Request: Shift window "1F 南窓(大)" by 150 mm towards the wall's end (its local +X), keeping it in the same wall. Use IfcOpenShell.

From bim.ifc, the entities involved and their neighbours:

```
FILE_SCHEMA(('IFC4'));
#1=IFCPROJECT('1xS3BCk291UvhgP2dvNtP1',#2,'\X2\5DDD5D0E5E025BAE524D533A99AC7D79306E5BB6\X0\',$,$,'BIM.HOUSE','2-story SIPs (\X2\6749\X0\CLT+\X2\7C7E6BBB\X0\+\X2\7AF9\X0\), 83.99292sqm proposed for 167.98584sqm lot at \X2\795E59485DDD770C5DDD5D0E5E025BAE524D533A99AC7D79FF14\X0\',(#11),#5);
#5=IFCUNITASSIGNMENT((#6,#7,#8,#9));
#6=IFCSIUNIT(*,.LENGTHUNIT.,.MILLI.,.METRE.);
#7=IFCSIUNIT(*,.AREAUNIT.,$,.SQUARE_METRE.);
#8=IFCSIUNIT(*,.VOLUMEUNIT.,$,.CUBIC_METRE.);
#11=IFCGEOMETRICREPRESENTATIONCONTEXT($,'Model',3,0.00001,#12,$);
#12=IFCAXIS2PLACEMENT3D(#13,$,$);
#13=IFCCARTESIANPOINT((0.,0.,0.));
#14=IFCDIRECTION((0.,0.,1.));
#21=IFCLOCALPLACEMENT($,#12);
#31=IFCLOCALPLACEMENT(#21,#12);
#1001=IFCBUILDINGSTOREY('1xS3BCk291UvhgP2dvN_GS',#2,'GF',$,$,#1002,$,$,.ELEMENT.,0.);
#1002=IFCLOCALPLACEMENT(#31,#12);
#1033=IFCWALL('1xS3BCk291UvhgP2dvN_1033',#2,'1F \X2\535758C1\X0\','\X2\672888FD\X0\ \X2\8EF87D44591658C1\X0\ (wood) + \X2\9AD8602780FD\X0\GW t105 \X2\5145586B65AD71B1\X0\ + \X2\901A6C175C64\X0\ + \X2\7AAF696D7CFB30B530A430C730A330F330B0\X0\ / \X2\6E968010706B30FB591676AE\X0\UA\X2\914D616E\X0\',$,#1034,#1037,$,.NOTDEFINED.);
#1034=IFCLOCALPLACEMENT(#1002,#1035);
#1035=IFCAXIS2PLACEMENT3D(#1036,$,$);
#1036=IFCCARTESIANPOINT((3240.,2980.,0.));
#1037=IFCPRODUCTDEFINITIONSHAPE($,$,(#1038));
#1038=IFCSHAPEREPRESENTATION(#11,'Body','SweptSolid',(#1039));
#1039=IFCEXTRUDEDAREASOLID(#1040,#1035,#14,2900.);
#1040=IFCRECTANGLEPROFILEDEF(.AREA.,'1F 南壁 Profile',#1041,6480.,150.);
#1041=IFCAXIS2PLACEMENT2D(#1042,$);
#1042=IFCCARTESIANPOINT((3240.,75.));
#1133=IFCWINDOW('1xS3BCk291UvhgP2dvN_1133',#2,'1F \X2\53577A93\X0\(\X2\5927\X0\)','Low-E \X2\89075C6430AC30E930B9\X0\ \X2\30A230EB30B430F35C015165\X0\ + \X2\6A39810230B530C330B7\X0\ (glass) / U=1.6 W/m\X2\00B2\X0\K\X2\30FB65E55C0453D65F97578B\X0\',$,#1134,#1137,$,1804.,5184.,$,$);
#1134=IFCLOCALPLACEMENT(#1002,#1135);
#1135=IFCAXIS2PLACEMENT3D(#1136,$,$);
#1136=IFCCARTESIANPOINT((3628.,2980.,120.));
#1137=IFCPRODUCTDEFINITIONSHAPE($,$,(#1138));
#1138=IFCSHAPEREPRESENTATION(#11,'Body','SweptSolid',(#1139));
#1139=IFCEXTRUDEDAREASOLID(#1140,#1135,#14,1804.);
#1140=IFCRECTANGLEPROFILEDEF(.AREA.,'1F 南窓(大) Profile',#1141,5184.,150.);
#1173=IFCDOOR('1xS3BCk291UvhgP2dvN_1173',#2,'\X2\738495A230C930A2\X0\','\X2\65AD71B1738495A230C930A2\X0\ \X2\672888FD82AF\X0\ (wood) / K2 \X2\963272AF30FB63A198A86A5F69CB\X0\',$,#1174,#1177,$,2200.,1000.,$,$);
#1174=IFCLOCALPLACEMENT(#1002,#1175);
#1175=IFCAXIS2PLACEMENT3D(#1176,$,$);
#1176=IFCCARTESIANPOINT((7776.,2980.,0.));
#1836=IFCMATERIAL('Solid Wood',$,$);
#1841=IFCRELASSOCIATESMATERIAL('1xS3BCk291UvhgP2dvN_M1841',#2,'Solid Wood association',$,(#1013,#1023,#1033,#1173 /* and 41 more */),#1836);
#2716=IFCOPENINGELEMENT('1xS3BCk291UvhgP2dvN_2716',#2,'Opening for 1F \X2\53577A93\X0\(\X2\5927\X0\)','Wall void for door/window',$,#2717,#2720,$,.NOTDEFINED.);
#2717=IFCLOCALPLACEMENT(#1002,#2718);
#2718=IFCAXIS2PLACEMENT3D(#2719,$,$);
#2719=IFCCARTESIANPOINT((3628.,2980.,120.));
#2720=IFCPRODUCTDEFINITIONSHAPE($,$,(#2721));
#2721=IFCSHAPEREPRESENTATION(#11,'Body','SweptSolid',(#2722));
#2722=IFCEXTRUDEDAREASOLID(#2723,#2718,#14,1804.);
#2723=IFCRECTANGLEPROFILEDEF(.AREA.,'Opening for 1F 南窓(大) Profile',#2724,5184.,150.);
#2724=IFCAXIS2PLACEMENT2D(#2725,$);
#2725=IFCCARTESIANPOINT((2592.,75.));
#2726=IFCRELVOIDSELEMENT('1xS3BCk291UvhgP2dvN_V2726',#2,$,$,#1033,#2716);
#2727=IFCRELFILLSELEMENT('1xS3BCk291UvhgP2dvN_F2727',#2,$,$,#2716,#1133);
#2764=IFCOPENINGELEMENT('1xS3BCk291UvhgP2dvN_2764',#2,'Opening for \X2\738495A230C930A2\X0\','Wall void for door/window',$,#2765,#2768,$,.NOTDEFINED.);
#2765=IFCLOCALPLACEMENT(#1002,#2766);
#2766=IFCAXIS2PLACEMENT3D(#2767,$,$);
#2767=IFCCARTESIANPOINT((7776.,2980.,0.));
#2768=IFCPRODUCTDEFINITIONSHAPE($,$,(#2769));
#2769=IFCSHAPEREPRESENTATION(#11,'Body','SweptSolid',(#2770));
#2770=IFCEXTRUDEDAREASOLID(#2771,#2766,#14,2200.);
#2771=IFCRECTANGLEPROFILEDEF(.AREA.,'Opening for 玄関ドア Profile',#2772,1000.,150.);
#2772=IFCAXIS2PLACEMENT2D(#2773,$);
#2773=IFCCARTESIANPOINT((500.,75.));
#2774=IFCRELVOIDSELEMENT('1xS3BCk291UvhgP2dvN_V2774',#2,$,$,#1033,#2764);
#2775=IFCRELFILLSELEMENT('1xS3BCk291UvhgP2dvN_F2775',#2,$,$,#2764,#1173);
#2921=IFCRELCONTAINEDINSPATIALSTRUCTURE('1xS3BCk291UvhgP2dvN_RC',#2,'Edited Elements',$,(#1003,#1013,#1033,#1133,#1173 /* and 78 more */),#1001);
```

```python
import ifcopenshell
import ifcopenshell.api.geometry
import ifcopenshell.util.placement
import ifcopenshell.util.unit

model = ifcopenshell.open("bim.ifc")
unit_scale = ifcopenshell.util.unit.calculate_unit_scale(model)

window = model.by_guid("1xS3BCk291UvhgP2dvN_1133")
opening = window.FillsVoids[0].RelatingOpeningElement
wall = opening.VoidsElements[0].RelatingBuildingElement

wall_matrix = ifcopenshell.util.placement.get_local_placement(wall.ObjectPlacement)
shift = wall_matrix[:3, 0] * 0.15 / unit_scale
before = ifcopenshell.util.placement.get_local_placement(window.ObjectPlacement)[:3, 3].copy()

# The window is not placed relative to its opening, so move both.
for product in (opening, window):
    matrix = ifcopenshell.util.placement.get_local_placement(product.ObjectPlacement)
    matrix[:3, 3] += shift
    ifcopenshell.api.geometry.edit_object_placement(model, product=product, matrix=matrix, is_si=False)

after = ifcopenshell.util.placement.get_local_placement(window.ObjectPlacement)[:3, 3]
print("window moved by", (after - before).round(3) + 0.0)

model.write("bim_updated.ifc")
```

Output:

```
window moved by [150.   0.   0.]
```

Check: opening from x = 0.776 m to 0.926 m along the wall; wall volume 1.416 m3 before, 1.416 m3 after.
